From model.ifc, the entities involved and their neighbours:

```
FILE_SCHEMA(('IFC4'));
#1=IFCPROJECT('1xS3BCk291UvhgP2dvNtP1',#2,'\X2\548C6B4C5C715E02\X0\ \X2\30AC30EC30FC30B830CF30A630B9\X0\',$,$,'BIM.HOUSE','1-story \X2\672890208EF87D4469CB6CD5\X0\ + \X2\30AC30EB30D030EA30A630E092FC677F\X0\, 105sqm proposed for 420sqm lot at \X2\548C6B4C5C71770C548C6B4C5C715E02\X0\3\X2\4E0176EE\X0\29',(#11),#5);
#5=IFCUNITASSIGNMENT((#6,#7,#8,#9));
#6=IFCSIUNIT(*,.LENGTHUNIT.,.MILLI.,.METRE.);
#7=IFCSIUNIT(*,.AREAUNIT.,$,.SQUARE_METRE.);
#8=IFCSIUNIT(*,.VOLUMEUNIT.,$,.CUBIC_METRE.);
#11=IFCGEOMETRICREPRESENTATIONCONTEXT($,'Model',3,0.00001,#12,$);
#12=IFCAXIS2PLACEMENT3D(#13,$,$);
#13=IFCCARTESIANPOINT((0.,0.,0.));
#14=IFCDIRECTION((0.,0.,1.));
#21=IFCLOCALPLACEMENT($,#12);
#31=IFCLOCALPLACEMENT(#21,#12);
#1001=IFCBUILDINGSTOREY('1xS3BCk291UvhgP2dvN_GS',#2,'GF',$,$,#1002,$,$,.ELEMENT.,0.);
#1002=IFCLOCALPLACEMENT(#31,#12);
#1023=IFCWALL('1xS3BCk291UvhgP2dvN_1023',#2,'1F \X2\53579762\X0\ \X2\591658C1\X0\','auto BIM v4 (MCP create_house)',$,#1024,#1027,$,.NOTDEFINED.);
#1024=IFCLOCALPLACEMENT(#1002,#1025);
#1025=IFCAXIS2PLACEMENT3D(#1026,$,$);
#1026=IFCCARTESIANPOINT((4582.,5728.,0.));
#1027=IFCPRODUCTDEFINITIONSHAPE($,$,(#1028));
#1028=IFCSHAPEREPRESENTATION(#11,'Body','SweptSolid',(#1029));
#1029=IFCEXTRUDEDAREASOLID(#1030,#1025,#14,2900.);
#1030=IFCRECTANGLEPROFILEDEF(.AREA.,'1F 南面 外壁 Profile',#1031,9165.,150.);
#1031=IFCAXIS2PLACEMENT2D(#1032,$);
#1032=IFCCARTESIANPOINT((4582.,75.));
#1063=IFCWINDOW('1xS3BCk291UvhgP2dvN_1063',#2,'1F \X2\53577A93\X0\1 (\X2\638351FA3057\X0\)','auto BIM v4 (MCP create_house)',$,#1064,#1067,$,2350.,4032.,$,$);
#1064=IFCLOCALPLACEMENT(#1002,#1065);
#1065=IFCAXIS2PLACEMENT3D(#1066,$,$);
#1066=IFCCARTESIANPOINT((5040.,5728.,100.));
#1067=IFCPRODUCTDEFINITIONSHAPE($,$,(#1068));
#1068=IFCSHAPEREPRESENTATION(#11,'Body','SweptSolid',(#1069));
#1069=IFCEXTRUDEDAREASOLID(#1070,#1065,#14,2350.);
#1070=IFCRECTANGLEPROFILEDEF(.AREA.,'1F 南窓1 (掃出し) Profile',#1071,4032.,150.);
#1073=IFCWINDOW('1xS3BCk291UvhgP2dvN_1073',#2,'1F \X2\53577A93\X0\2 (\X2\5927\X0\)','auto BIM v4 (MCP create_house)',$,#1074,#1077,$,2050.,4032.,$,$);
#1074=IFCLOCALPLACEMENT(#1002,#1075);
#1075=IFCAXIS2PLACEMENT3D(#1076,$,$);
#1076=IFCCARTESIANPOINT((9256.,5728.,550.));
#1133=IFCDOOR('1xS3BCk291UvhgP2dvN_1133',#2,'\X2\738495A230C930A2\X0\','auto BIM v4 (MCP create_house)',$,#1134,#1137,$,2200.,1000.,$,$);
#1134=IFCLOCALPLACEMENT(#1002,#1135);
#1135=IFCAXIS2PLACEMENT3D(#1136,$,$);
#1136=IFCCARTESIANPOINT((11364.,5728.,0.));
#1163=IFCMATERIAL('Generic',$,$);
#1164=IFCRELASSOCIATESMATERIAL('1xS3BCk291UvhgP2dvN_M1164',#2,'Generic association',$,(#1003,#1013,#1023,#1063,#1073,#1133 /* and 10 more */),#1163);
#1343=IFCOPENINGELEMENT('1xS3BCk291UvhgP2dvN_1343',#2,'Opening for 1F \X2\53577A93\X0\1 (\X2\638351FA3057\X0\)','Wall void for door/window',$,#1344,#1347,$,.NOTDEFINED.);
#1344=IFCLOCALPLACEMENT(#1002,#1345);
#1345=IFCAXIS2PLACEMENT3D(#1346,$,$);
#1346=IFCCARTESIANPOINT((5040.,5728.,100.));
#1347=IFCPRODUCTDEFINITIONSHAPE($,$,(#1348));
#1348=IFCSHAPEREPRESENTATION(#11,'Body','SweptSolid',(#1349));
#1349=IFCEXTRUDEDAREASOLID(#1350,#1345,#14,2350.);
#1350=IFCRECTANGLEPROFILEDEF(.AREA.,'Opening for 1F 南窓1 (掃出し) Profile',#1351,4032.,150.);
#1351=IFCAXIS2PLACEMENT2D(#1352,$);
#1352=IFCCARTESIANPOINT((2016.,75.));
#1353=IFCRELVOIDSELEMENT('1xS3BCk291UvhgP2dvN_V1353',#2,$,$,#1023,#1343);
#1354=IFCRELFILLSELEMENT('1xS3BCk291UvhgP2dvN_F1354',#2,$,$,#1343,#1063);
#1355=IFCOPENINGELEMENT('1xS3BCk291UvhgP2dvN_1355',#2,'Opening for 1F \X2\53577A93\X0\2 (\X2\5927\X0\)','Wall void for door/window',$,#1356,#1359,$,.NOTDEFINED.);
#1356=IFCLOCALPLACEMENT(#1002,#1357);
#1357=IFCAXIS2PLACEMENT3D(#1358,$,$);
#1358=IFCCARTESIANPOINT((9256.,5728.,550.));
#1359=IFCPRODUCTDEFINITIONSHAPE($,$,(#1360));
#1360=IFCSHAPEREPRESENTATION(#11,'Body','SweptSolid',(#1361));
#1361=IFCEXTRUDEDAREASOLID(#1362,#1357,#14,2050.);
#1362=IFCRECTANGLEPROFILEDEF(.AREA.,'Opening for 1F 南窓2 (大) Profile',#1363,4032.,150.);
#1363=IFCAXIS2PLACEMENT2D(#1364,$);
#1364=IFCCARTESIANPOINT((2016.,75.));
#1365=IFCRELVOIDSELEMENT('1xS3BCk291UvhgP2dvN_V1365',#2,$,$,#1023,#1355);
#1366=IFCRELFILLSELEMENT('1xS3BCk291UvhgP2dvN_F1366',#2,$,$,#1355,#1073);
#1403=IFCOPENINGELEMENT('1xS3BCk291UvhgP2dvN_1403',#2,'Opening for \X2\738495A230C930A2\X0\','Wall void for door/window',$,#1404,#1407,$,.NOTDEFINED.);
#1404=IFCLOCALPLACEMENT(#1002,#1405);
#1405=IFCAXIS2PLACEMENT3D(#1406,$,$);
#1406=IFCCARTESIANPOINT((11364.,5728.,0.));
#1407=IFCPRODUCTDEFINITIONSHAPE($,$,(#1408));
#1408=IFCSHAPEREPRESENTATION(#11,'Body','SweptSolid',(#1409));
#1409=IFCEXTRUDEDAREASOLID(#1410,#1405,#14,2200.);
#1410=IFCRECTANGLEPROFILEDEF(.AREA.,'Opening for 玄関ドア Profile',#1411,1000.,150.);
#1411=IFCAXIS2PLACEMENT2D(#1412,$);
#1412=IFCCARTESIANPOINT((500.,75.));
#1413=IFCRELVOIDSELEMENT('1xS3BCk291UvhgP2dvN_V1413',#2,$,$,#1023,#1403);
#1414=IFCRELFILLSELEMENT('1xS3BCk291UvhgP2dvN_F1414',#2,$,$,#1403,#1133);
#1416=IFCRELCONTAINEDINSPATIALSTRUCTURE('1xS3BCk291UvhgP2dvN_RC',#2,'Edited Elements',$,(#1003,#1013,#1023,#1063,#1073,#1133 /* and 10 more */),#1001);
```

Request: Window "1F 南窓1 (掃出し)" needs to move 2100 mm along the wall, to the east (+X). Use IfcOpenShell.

```python
import ifcopenshell
import ifcopenshell.api.geometry
import ifcopenshell.util.placement

model = ifcopenshell.open("model.ifc")

window = model.by_id(1063)
opening = window.FillsVoids[0].RelatingOpeningElement
wall = opening.VoidsElements[0].RelatingBuildingElement

wall_matrix = ifcopenshell.util.placement.get_local_placement(wall.ObjectPlacement)
shift = wall_matrix[:3, 0] * 2100.0
before = ifcopenshell.util.placement.get_local_placement(window.ObjectPlacement)[:3, 3].copy()

# The window is not placed relative to its opening, so move both.
for product in (opening, window):
    matrix = ifcopenshell.util.placement.get_local_placement(product.ObjectPlacement)
    matrix[:3, 3] += shift
    ifcopenshell.api.geometry.edit_object_placement(model, product=product, matrix=matrix, is_si=False)

after = ifcopenshell.util.placement.get_local_placement(window.ObjectPlacement)[:3, 3]
print("window moved by", (after - before).round(3) + 0.0)

model.write("model_v2.ifc")
```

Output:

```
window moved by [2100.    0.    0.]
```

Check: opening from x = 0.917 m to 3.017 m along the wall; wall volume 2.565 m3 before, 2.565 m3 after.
